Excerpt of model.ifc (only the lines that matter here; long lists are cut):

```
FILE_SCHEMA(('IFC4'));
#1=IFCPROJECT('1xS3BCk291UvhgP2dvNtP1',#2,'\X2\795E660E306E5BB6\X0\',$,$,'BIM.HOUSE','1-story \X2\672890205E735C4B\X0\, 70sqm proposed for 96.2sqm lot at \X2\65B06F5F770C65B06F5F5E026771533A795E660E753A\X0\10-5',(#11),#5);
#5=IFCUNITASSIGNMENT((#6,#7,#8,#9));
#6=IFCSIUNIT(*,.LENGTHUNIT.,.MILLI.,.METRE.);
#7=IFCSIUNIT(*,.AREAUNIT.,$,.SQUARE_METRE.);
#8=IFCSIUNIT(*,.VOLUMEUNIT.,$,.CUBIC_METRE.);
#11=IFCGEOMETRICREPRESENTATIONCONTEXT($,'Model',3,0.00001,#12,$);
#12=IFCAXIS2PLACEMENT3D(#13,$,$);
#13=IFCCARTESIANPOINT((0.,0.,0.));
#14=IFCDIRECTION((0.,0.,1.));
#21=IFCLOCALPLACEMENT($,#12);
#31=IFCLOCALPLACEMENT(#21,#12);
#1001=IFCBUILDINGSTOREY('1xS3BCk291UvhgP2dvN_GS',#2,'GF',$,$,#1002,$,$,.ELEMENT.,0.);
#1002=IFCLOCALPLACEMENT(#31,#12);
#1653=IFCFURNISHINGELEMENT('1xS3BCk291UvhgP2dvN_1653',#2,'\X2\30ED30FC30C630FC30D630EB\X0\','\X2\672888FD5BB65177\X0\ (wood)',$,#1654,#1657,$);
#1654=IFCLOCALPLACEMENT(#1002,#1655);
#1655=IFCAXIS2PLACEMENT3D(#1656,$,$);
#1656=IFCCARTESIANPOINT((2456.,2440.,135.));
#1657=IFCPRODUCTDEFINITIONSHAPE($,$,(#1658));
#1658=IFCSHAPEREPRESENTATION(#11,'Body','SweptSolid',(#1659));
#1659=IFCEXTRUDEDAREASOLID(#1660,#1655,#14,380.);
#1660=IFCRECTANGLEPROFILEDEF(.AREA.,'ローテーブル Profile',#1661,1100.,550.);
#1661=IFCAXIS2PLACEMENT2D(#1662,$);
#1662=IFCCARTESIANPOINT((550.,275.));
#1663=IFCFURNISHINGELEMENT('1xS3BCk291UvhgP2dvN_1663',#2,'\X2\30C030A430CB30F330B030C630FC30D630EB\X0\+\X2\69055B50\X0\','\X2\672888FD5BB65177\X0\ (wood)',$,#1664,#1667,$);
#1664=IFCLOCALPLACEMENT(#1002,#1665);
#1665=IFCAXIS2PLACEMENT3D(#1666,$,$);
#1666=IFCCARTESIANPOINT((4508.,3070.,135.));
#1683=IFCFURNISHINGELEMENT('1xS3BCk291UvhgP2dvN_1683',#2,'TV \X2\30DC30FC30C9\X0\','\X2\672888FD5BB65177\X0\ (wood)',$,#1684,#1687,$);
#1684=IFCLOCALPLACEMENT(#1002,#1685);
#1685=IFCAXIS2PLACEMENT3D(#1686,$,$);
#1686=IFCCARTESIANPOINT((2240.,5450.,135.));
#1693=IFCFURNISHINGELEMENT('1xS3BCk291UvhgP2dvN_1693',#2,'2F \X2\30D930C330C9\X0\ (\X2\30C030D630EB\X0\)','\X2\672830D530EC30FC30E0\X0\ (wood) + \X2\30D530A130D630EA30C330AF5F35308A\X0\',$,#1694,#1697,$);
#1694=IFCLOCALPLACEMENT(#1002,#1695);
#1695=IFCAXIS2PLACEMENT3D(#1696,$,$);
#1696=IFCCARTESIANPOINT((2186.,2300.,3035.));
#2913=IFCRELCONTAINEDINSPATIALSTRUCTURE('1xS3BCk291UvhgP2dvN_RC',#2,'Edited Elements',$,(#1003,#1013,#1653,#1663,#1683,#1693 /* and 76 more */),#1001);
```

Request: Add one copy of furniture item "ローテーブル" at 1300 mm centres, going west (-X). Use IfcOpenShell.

```python
import numpy as np
import ifcopenshell
import ifcopenshell.api.geometry
import ifcopenshell.api.root
import ifcopenshell.util.element
import ifcopenshell.util.placement

model = ifcopenshell.open("model.ifc")


def reuse_history(source, copy):
    """copy_class also copies each property set's owner history, people and application; keep the originals."""
    for rel in copy.IsDefinedBy:
        if rel.is_a("IfcRelDefinesByProperties") and (history := rel.RelatingPropertyDefinition.OwnerHistory):
            rel.RelatingPropertyDefinition.OwnerHistory = source.OwnerHistory
            ifcopenshell.util.element.remove_deep2(model, history)


source = model.by_guid("1xS3BCk291UvhgP2dvN_1653")
base = ifcopenshell.util.placement.get_local_placement(source.ObjectPlacement)
step = np.array([-1.0, 0.0, 0.0]) * 1300.0

for i in range(1, 2):
    copy = ifcopenshell.api.root.copy_class(model, product=source)
    copy.Representation = ifcopenshell.util.element.copy_deep(
        model, source.Representation, exclude=["IfcGeometricRepresentationContext", "IfcRepresentationMap"]
    )
    reuse_history(source, copy)
    matrix = base.copy()
    matrix[:3, 3] += i * step
    print("added at", matrix[:3, 3].round(3) + 0.0)
    ifcopenshell.api.geometry.edit_object_placement(model, product=copy, matrix=matrix, is_si=False)

model.write("model-out.ifc")
```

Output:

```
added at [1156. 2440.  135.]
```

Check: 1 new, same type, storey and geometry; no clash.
